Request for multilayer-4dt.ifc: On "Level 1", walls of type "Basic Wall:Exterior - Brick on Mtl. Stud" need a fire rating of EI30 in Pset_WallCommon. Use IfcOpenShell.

First a look at what the model holds.

```python
import ifcopenshell
import ifcopenshell.util.element

model = ifcopenshell.open("multilayer-4dt.ifc")
print(model.schema)
storey = next(s for s in model.by_type("IfcBuildingStorey") if s.Name == "Level 1")
walls = [e for e in ifcopenshell.util.element.get_decomposition(storey) if e.is_a("IfcWall")]
seen = {}
for e in walls:
    element_type = ifcopenshell.util.element.get_type(e)
    key = (element_type.Name if element_type != e and element_type else None, ifcopenshell.util.element.get_pset(e, "Pset_WallCommon", "FireRating"))
    seen[key] = seen.get(key, 0) + 1
for (name, value), count in sorted(seen.items(), key=str):
    print(count, "x", name, "|", value)
```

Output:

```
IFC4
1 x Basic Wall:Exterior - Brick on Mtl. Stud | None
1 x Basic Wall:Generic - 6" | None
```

```python
import ifcopenshell
import ifcopenshell.api.pset
import ifcopenshell.util.element

model = ifcopenshell.open("multilayer-4dt.ifc")

storey = next(s for s in model.by_type("IfcBuildingStorey") if s.Name == "Level 1")
walls = [e for e in ifcopenshell.util.element.get_decomposition(storey) if e.is_a("IfcWall")]

count = 0
for e in walls:
    element_type = ifcopenshell.util.element.get_type(e)
    if element_type in (None, e) or element_type.Name != "Basic Wall:Exterior - Brick on Mtl. Stud":
        continue
    # add_pset returns the element's existing set when there is one.
    pset = ifcopenshell.api.pset.add_pset(model, product=e, name="Pset_WallCommon")
    ifcopenshell.api.pset.edit_pset(model, pset=pset, properties={"FireRating": "EI30"})
    count += 1

print(count, "walls updated")

model.write("multilayer-4dt_edited.ifc")
```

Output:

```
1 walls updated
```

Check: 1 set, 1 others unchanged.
